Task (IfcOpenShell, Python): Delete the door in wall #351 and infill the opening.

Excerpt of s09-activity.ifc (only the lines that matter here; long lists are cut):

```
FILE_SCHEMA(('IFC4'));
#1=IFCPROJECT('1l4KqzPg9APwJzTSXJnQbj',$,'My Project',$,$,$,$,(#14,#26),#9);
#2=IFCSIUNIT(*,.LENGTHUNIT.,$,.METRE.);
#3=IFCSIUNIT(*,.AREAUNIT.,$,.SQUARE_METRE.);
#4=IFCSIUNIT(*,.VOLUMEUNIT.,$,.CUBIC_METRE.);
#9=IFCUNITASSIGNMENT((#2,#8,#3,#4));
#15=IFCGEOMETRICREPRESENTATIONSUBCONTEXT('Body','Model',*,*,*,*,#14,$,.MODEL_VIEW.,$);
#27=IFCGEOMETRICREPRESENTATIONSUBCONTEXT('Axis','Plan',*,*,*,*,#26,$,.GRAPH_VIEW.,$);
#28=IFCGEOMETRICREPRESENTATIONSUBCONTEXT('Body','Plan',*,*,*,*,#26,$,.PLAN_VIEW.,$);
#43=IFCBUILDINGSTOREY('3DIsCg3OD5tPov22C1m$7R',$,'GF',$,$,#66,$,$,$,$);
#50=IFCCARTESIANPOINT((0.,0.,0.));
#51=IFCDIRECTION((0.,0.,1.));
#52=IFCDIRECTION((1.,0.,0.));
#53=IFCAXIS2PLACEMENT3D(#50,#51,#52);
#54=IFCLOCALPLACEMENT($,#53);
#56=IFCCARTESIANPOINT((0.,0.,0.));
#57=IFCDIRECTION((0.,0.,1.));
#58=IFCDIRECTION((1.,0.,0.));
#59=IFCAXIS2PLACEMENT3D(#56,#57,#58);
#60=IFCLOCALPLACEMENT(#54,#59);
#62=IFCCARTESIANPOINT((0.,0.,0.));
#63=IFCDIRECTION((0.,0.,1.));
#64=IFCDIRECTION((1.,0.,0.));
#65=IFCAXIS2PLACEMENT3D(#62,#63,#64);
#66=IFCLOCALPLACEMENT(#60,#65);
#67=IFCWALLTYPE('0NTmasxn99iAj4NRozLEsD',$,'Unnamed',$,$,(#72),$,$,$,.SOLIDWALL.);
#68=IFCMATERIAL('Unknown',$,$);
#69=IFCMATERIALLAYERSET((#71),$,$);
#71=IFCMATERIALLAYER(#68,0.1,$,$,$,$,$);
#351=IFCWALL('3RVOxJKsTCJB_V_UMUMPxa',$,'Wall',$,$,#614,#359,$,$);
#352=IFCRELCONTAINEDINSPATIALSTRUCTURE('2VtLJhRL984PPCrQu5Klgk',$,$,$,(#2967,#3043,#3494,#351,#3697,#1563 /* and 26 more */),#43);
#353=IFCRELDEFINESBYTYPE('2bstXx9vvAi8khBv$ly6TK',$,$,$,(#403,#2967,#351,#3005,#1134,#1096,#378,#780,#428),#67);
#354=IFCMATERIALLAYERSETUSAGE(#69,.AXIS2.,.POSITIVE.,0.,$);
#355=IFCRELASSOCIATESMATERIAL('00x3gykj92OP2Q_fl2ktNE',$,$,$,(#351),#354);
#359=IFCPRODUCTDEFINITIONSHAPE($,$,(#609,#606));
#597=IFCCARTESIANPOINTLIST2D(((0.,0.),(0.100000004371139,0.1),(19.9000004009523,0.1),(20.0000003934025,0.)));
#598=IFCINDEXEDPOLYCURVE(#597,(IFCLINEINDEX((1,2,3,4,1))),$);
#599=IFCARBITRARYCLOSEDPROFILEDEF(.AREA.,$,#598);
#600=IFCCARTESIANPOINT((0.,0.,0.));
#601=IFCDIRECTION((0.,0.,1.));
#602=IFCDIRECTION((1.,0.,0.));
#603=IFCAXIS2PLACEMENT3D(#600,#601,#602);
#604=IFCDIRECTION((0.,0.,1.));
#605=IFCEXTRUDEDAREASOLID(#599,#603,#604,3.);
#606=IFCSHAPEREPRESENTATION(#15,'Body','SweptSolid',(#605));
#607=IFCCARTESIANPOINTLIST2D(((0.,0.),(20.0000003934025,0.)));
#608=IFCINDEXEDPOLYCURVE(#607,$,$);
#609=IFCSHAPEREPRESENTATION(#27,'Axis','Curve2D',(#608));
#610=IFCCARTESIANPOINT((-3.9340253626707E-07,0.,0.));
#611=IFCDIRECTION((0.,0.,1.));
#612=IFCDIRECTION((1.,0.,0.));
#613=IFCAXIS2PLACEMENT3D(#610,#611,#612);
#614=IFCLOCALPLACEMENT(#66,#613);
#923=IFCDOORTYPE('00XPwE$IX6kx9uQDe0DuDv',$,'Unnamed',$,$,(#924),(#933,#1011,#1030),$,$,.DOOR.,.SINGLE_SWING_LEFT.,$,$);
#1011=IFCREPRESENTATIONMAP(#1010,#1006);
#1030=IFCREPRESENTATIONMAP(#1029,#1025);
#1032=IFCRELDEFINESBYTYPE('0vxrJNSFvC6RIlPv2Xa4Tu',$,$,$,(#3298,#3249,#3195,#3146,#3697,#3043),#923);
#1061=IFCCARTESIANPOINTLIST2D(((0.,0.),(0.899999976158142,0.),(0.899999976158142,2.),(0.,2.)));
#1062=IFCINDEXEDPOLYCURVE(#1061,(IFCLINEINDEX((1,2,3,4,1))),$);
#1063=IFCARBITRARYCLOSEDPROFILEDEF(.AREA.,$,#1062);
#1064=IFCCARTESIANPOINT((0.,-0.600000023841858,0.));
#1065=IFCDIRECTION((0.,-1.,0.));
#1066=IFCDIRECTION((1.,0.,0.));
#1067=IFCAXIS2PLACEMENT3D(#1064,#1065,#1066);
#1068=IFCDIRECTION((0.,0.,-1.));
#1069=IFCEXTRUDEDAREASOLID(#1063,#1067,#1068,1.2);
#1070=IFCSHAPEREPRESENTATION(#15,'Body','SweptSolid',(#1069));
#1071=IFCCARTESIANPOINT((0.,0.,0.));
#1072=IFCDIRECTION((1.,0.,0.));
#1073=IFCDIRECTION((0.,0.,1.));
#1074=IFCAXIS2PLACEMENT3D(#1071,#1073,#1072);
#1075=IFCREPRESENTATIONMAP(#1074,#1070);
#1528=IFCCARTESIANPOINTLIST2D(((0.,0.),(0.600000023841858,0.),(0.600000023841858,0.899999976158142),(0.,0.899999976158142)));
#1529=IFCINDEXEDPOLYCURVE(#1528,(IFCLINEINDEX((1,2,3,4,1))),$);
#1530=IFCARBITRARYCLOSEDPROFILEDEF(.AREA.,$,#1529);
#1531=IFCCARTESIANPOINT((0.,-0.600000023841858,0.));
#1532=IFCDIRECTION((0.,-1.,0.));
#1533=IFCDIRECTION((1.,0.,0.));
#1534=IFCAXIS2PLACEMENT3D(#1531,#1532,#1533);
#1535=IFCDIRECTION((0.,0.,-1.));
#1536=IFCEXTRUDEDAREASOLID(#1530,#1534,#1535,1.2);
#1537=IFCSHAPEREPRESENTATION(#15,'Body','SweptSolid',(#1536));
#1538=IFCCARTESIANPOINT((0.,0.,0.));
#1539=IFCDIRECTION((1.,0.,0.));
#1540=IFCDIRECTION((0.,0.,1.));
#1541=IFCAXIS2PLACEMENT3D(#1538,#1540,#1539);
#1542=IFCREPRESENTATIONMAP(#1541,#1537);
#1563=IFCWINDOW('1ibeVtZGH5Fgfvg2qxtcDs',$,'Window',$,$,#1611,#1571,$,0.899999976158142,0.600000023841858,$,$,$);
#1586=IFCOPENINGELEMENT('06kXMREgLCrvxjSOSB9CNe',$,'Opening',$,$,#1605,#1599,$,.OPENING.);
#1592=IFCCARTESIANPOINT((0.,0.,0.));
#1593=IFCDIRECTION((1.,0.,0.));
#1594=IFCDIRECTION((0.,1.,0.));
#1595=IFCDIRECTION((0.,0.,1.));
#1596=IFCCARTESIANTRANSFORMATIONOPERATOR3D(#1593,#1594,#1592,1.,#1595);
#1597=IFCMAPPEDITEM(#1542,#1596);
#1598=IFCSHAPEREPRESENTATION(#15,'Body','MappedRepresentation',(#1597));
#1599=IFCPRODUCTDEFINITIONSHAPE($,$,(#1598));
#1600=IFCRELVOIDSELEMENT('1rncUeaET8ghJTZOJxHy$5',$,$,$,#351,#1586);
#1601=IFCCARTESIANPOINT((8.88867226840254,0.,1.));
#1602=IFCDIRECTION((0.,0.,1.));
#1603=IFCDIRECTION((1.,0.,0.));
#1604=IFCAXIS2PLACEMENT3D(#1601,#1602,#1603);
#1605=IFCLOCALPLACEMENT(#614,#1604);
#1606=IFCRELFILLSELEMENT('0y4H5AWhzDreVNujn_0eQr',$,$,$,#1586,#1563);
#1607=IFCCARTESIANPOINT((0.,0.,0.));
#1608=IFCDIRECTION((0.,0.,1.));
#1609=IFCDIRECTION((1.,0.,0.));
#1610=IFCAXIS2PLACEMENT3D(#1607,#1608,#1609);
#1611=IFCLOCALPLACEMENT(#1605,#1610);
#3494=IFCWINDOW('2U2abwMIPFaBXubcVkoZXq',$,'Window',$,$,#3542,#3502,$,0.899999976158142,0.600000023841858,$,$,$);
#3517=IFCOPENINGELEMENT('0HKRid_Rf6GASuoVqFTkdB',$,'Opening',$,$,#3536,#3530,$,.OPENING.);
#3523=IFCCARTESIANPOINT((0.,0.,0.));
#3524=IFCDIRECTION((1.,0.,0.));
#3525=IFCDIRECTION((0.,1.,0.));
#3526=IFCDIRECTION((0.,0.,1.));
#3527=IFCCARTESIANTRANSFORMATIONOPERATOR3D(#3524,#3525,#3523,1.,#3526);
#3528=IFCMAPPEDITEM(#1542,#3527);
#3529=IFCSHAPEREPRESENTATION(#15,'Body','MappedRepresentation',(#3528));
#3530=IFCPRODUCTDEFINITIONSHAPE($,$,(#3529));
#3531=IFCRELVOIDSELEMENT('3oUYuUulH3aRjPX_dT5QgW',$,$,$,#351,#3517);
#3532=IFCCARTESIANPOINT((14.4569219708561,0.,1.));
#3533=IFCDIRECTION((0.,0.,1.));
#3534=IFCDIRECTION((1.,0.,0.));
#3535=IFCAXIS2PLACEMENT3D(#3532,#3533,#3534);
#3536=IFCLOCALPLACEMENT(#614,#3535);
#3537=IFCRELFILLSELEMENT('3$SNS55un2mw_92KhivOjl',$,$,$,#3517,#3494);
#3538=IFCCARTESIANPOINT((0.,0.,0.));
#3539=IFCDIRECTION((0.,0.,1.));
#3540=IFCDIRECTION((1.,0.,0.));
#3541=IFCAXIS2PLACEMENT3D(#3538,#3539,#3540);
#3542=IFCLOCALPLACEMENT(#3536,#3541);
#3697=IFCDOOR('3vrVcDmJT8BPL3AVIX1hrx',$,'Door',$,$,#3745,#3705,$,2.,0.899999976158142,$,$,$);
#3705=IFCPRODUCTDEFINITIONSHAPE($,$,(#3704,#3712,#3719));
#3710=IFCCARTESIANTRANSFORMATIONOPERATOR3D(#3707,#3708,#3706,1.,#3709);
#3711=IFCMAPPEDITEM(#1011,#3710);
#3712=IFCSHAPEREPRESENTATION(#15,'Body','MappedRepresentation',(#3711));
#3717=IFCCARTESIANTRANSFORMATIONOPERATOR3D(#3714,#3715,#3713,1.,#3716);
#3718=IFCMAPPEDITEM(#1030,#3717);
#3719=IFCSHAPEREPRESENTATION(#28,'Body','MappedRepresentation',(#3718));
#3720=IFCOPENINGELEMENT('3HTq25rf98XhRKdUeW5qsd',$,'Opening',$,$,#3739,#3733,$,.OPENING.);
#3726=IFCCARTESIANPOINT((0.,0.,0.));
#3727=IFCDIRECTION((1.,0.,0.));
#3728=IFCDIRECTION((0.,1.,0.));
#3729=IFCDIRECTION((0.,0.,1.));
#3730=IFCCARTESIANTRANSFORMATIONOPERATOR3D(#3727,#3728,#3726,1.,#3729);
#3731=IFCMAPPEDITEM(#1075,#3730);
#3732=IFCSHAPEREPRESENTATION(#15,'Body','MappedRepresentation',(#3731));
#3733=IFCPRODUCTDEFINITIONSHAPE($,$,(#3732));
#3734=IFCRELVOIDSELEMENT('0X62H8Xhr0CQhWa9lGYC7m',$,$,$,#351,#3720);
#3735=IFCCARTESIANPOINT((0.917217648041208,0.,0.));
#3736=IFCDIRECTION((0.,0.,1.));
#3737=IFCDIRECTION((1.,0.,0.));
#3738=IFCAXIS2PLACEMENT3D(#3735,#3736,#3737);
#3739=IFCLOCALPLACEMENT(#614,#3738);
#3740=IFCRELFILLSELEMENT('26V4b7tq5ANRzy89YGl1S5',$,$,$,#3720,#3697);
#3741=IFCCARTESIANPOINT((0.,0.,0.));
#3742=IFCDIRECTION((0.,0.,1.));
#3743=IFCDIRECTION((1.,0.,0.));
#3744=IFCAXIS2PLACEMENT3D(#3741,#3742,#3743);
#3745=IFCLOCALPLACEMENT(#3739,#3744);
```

```python
import ifcopenshell
import ifcopenshell.api.feature
import ifcopenshell.api.root
import ifcopenshell.geom
import ifcopenshell.util.shape

model = ifcopenshell.open("s09-activity.ifc")
settings = ifcopenshell.geom.settings()


def volume(element):
    """Net volume in cubic metres, openings subtracted."""
    shape = ifcopenshell.geom.create_shape(settings, element)
    return ifcopenshell.util.shape.get_volume(shape.geometry)


door = model.by_id(3697)
opening = door.FillsVoids[0].RelatingOpeningElement
wall = opening.VoidsElements[0].RelatingBuildingElement
before = volume(wall)

ifcopenshell.api.root.remove_product(model, product=door)
ifcopenshell.api.feature.remove_feature(model, feature=opening)

after = volume(wall)

print(f"wall volume {before:.3f} -> {after:.3f} m3")

model.write("s09-activity_edited.ifc")
```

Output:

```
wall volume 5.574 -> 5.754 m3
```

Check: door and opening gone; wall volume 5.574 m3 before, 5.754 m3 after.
